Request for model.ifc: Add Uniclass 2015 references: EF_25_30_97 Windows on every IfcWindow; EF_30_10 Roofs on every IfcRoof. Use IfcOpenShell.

First a look at what the model holds.

```python
import ifcopenshell

model = ifcopenshell.open("model.ifc")
print(model.schema)
print("classifications:", [c.Name for c in model.by_type("IfcClassification")])
for ifc_class in ("IfcDoor", "IfcRoof", "IfcStair", "IfcWall", "IfcWindow"):
    print(ifc_class, len(model.by_type(ifc_class)))
```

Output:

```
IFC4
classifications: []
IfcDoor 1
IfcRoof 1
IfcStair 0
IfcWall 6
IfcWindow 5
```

```python
import ifcopenshell
import ifcopenshell.api.classification

model = ifcopenshell.open("model.ifc")

system = ifcopenshell.api.classification.add_classification(model, classification="Uniclass 2015")

codes = {
    "IfcWindow": ("EF_25_30_97", "Windows"),
    "IfcRoof": ("EF_30_10", "Roofs"),
}
for ifc_class, (code, name) in codes.items():
    products = model.by_type(ifc_class)
    ifcopenshell.api.classification.add_reference(
        model, products=products, classification=system, identification=code, name=name
    )
    print(code, len(products))

model.write("model_v2.ifc")
```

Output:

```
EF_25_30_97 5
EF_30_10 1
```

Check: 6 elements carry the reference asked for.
